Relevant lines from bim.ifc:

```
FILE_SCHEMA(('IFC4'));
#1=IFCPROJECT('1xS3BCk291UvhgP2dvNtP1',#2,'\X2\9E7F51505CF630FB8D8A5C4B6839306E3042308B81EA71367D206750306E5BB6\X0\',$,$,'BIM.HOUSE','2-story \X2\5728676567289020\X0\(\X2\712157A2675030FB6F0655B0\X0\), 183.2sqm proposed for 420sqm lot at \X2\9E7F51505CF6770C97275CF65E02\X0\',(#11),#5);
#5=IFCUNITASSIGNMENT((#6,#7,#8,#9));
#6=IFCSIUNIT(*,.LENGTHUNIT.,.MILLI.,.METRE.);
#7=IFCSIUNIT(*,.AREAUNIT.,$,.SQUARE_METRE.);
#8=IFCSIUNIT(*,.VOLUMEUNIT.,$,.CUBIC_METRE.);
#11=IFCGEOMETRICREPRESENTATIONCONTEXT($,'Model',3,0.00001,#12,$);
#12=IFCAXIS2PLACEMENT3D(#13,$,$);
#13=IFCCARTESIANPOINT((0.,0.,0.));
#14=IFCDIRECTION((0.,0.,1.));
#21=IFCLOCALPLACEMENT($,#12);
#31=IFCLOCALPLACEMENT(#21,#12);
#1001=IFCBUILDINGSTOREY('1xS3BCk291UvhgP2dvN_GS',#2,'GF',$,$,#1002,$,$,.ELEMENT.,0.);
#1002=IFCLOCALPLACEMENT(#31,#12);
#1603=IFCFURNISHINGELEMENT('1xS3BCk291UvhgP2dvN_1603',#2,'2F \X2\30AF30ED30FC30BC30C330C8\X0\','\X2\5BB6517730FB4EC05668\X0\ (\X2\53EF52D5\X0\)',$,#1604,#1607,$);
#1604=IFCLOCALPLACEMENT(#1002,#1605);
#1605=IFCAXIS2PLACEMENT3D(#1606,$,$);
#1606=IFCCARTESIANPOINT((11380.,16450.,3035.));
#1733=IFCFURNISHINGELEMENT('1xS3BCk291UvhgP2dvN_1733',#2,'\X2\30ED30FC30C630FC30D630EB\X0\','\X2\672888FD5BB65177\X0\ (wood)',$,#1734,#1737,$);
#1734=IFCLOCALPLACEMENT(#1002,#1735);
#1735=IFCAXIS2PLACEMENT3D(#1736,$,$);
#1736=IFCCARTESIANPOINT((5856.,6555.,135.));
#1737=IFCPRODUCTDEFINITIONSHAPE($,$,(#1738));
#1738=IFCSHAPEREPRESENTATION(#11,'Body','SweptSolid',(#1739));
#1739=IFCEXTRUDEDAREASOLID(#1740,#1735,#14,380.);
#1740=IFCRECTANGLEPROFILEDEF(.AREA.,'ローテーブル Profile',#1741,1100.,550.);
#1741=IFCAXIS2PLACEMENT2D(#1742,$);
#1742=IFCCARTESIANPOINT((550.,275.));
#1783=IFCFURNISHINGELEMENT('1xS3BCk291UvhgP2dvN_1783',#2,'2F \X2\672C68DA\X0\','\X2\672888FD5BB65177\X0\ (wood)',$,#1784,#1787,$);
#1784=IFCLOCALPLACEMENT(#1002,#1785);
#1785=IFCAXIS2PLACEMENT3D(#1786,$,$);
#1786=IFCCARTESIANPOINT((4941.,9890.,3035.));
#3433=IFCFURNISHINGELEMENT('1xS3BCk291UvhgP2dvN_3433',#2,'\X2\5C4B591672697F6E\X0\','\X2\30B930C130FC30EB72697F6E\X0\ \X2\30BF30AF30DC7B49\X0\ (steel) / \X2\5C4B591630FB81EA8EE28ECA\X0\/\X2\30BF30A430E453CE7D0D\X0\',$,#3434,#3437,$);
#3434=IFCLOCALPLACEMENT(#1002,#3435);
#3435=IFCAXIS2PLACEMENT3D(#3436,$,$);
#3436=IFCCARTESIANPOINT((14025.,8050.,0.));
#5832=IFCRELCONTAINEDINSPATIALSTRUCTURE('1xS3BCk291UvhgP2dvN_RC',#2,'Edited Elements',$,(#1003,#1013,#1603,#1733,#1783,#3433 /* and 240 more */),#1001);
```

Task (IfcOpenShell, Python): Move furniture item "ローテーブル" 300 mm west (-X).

```python
import ifcopenshell
import ifcopenshell.api.geometry
import ifcopenshell.util.placement
import ifcopenshell.util.unit

model = ifcopenshell.open("bim.ifc")
unit_scale = ifcopenshell.util.unit.calculate_unit_scale(model)

item = model.by_guid("1xS3BCk291UvhgP2dvN_1733")
matrix = ifcopenshell.util.placement.get_local_placement(item.ObjectPlacement)
matrix[0, 3] -= 0.3 / unit_scale
ifcopenshell.api.geometry.edit_object_placement(model, product=item, matrix=matrix, is_si=False)

print(ifcopenshell.util.placement.get_local_placement(item.ObjectPlacement).round(3) + 0.0)

model.write("bim-out.ifc")
```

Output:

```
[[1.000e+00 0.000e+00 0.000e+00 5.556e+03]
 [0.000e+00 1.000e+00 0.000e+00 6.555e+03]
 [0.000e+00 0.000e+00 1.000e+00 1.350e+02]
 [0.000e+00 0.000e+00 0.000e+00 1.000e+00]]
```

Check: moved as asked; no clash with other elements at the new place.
